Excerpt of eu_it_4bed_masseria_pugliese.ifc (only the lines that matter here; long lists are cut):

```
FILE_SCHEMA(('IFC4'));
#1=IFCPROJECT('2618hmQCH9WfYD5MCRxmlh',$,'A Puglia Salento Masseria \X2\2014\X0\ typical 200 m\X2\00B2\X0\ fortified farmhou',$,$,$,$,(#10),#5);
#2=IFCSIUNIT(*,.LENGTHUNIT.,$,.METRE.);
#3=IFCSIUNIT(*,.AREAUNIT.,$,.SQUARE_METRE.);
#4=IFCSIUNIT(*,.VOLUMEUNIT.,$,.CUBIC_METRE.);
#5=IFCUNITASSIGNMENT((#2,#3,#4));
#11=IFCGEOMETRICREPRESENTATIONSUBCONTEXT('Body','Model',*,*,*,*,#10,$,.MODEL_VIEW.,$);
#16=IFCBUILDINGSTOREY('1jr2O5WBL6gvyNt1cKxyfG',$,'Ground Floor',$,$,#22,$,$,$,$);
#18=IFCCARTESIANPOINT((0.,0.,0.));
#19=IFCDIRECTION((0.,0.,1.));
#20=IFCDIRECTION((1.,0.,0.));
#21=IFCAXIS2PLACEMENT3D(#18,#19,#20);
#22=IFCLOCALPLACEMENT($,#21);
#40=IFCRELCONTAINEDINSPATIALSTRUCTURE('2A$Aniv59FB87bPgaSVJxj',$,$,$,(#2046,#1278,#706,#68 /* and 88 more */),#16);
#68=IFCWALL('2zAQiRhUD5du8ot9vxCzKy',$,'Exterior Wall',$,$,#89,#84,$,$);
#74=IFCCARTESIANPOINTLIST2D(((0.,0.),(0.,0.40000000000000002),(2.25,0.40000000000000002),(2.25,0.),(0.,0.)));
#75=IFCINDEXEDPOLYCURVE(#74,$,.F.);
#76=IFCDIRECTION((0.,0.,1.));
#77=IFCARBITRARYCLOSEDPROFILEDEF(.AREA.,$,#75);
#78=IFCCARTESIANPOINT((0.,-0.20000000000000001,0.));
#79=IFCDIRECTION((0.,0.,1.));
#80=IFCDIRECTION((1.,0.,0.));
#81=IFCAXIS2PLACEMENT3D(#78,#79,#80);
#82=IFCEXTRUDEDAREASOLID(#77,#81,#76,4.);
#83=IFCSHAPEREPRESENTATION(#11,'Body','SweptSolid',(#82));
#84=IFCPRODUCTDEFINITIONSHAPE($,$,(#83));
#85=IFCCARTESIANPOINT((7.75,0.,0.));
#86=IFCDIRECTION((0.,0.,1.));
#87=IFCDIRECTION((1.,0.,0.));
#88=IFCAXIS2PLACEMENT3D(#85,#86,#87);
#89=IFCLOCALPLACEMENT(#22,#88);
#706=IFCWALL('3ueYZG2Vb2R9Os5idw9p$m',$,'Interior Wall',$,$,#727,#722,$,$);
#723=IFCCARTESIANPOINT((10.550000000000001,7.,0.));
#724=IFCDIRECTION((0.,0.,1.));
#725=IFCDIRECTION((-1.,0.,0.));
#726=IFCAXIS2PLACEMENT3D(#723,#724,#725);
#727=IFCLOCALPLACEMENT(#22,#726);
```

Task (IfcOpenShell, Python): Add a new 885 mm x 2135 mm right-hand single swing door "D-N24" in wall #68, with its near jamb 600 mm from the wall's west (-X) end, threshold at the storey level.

```python
import numpy as np
import ifcopenshell
import ifcopenshell.api.feature
import ifcopenshell.api.geometry
import ifcopenshell.api.root
import ifcopenshell.api.spatial
import ifcopenshell.geom
import ifcopenshell.util.element
import ifcopenshell.util.placement
import ifcopenshell.util.representation
import ifcopenshell.util.shape
import ifcopenshell.util.unit

model = ifcopenshell.open("eu_it_4bed_masseria_pugliese.ifc")
unit_scale = ifcopenshell.util.unit.calculate_unit_scale(model)
settings = ifcopenshell.geom.settings()


def volume(element):
    """Net volume in cubic metres, openings subtracted."""
    shape = ifcopenshell.geom.create_shape(settings, element)
    return ifcopenshell.util.shape.get_volume(shape.geometry)


wall = model.by_guid("2zAQiRhUD5du8ot9vxCzKy")
storey = ifcopenshell.util.element.get_container(wall, ifc_class="IfcBuildingStorey")
context = ifcopenshell.util.representation.get_context(model, "Model", "Body", "MODEL_VIEW")
before = volume(wall)

width, height, from_end, sill = 0.885, 2.135, 0.6, 0.0  # metres

# The wall runs along its own X axis, and the end named is its -X end.
wall_shape = ifcopenshell.geom.create_shape(settings, wall)
x, y, z = ifcopenshell.util.shape.get_vertices(wall_shape.geometry).T
start = x.min() + from_end
face, thickness = float(y.min()), float(y.max() - y.min())
wall_matrix = ifcopenshell.util.placement.get_local_placement(wall.ObjectPlacement)
level = ifcopenshell.util.placement.get_local_placement(storey.ObjectPlacement)[2, 3]


def in_wall(x, y):
    """Placement at x, y metres in the wall's axes, at sill height."""
    matrix = wall_matrix.copy()
    matrix[:, 3] = wall_matrix @ np.array([x / unit_scale, y / unit_scale, 0.0, 1.0])
    matrix[2, 3] = level + sill / unit_scale
    return matrix


# Opening: a box that overshoots both wall faces by 50 mm.
opening = ifcopenshell.api.root.create_entity(model, ifc_class="IfcOpeningElement", predefined_type="OPENING")
box = ifcopenshell.api.geometry.add_wall_representation(
    model, context=context, length=width, height=height, thickness=thickness + 0.1
)
ifcopenshell.api.geometry.assign_representation(model, product=opening, representation=box)
ifcopenshell.api.geometry.edit_object_placement(model, product=opening, matrix=in_wall(start, face - 0.05), is_si=False)
ifcopenshell.api.feature.add_feature(model, feature=opening, element=wall)

door = ifcopenshell.api.root.create_entity(model, ifc_class="IfcDoor", name="D-N24", predefined_type="DOOR")
door.OverallWidth, door.OverallHeight = width / unit_scale, height / unit_scale
door.OperationType = "SINGLE_SWING_RIGHT"
body = ifcopenshell.api.geometry.add_door_representation(
    model,
    context=context,
    overall_width=door.OverallWidth,
    overall_height=door.OverallHeight,
    operation_type="SINGLE_SWING_RIGHT",
    lining_properties={"LiningDepth": thickness / unit_scale, "ThresholdDepth": thickness / unit_scale},
)
ifcopenshell.api.geometry.assign_representation(model, product=door, representation=body)
ifcopenshell.api.spatial.assign_container(model, products=[door], relating_structure=storey)
ifcopenshell.api.feature.add_filling(model, opening=opening, element=door)

# The lining spans the wall, so the door starts at the wall face.
ifcopenshell.api.geometry.edit_object_placement(model, product=door, matrix=in_wall(start, face), is_si=False)

after = volume(wall)

print(f"wall volume {before:.3f} -> {after:.3f} m3")

model.write("eu_it_4bed_masseria_pugliese-out.ifc")
```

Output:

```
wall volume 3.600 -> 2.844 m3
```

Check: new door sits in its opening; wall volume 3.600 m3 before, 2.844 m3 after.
